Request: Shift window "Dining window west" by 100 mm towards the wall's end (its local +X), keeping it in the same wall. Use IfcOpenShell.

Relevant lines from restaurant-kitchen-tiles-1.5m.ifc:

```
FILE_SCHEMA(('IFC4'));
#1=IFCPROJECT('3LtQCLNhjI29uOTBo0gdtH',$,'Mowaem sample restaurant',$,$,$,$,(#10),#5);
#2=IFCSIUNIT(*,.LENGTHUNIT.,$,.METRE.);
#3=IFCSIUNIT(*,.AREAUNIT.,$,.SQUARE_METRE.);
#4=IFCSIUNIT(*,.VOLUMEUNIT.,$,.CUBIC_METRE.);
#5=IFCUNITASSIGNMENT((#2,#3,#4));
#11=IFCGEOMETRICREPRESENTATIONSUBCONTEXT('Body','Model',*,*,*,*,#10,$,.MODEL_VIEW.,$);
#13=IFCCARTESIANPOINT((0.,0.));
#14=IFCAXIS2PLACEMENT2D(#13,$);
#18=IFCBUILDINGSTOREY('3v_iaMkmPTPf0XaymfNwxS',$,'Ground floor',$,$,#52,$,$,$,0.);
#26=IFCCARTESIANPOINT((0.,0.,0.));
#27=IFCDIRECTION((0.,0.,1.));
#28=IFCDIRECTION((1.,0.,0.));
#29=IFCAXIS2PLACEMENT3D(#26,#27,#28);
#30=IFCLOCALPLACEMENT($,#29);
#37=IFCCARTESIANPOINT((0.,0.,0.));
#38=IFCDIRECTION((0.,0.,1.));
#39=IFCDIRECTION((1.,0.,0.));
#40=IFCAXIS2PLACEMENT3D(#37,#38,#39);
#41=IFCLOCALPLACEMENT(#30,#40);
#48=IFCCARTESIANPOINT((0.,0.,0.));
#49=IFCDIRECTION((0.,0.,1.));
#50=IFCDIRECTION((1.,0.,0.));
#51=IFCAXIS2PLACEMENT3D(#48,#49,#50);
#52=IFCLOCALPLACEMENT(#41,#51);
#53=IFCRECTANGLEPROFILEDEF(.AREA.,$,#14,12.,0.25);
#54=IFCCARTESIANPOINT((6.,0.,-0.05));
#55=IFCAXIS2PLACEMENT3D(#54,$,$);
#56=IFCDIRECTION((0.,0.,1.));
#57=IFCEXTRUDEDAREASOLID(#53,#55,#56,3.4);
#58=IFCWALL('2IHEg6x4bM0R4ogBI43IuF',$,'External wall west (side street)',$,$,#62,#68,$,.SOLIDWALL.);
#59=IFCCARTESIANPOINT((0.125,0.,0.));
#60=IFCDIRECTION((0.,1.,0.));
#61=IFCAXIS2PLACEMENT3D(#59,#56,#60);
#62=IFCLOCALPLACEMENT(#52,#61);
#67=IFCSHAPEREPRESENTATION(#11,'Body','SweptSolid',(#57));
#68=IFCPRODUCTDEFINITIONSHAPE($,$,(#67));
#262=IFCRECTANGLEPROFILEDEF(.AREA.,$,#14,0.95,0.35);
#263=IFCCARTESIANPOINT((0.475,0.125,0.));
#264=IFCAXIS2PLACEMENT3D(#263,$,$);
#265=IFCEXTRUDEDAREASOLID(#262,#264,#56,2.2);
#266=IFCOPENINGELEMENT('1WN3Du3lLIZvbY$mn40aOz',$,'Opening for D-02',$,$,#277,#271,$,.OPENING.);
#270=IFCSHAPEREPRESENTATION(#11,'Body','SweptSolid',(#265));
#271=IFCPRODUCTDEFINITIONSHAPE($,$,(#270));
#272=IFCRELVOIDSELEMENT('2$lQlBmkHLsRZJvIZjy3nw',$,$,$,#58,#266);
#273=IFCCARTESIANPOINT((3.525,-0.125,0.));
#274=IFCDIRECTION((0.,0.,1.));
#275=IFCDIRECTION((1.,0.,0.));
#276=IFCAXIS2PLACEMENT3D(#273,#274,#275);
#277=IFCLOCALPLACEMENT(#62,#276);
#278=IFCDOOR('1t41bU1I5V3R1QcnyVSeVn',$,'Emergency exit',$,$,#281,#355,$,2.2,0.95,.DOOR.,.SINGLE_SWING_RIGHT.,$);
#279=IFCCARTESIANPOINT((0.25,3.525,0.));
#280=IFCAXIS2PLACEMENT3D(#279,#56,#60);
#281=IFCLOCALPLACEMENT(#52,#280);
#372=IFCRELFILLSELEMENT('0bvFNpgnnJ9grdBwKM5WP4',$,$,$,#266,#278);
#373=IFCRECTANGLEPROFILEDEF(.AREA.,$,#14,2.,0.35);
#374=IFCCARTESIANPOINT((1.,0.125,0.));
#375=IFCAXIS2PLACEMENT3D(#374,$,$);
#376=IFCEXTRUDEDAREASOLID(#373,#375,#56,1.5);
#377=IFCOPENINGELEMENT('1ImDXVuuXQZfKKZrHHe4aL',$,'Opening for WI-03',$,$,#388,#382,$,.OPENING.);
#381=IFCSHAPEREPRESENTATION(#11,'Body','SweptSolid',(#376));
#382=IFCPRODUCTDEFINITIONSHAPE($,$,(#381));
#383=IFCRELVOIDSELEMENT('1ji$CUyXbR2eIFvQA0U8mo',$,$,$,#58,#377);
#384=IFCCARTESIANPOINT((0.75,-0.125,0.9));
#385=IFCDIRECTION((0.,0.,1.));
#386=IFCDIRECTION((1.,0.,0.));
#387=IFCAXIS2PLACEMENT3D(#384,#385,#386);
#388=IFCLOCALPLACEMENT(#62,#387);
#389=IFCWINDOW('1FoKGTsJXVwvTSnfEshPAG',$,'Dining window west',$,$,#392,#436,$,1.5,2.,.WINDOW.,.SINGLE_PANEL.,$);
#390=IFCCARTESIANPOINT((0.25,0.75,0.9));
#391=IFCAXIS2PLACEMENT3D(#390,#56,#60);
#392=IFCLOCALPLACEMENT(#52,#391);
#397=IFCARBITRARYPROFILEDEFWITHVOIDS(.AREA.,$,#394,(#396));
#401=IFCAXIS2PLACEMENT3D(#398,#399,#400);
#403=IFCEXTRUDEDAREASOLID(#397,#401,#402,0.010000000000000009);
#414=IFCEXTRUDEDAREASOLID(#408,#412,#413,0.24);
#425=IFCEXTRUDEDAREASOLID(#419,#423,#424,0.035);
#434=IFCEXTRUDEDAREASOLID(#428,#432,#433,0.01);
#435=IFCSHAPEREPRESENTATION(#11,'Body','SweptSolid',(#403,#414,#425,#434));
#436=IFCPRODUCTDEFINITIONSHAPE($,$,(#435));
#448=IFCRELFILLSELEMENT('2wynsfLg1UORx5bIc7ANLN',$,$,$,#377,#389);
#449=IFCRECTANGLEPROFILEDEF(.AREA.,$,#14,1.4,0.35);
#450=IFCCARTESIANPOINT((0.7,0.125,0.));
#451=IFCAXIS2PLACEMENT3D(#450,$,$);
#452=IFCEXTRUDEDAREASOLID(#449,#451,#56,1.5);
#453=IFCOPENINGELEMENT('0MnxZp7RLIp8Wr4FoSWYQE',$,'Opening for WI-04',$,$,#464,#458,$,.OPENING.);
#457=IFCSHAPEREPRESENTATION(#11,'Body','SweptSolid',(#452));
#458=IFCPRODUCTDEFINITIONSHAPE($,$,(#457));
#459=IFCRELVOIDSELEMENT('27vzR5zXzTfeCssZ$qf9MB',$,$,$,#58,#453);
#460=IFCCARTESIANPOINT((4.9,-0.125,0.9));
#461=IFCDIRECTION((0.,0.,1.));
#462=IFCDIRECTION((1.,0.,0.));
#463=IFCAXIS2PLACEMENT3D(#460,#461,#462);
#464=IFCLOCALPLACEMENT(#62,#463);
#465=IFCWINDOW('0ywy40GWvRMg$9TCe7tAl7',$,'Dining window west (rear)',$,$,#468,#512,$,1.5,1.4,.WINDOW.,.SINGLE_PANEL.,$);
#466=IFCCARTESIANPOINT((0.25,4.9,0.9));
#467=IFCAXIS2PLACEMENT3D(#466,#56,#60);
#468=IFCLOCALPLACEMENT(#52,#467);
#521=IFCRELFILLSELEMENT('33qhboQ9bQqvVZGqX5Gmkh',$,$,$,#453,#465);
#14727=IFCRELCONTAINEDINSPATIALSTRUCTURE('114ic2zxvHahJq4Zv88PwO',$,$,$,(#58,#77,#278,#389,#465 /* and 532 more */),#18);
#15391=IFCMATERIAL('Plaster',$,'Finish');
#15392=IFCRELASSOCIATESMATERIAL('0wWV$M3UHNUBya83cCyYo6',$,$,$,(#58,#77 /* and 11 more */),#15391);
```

```python
import ifcopenshell
import ifcopenshell.api.geometry
import ifcopenshell.util.placement
import ifcopenshell.util.unit

model = ifcopenshell.open("restaurant-kitchen-tiles-1.5m.ifc")
unit_scale = ifcopenshell.util.unit.calculate_unit_scale(model)

window = model.by_guid("1FoKGTsJXVwvTSnfEshPAG")
opening = window.FillsVoids[0].RelatingOpeningElement
wall = opening.VoidsElements[0].RelatingBuildingElement

wall_matrix = ifcopenshell.util.placement.get_local_placement(wall.ObjectPlacement)
shift = wall_matrix[:3, 0] * 0.1 / unit_scale
before = ifcopenshell.util.placement.get_local_placement(window.ObjectPlacement)[:3, 3].copy()

# The window is not placed relative to its opening, so move both.
for product in (opening, window):
    matrix = ifcopenshell.util.placement.get_local_placement(product.ObjectPlacement)
    matrix[:3, 3] += shift
    ifcopenshell.api.geometry.edit_object_placement(model, product=product, matrix=matrix, is_si=False)

after = ifcopenshell.util.placement.get_local_placement(window.ObjectPlacement)[:3, 3]
print("window moved by", (after - before).round(3) + 0.0)

model.write("restaurant-kitchen-tiles-1.5m_v2.ifc")
```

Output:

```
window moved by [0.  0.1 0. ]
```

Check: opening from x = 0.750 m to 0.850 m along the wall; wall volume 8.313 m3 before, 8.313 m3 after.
